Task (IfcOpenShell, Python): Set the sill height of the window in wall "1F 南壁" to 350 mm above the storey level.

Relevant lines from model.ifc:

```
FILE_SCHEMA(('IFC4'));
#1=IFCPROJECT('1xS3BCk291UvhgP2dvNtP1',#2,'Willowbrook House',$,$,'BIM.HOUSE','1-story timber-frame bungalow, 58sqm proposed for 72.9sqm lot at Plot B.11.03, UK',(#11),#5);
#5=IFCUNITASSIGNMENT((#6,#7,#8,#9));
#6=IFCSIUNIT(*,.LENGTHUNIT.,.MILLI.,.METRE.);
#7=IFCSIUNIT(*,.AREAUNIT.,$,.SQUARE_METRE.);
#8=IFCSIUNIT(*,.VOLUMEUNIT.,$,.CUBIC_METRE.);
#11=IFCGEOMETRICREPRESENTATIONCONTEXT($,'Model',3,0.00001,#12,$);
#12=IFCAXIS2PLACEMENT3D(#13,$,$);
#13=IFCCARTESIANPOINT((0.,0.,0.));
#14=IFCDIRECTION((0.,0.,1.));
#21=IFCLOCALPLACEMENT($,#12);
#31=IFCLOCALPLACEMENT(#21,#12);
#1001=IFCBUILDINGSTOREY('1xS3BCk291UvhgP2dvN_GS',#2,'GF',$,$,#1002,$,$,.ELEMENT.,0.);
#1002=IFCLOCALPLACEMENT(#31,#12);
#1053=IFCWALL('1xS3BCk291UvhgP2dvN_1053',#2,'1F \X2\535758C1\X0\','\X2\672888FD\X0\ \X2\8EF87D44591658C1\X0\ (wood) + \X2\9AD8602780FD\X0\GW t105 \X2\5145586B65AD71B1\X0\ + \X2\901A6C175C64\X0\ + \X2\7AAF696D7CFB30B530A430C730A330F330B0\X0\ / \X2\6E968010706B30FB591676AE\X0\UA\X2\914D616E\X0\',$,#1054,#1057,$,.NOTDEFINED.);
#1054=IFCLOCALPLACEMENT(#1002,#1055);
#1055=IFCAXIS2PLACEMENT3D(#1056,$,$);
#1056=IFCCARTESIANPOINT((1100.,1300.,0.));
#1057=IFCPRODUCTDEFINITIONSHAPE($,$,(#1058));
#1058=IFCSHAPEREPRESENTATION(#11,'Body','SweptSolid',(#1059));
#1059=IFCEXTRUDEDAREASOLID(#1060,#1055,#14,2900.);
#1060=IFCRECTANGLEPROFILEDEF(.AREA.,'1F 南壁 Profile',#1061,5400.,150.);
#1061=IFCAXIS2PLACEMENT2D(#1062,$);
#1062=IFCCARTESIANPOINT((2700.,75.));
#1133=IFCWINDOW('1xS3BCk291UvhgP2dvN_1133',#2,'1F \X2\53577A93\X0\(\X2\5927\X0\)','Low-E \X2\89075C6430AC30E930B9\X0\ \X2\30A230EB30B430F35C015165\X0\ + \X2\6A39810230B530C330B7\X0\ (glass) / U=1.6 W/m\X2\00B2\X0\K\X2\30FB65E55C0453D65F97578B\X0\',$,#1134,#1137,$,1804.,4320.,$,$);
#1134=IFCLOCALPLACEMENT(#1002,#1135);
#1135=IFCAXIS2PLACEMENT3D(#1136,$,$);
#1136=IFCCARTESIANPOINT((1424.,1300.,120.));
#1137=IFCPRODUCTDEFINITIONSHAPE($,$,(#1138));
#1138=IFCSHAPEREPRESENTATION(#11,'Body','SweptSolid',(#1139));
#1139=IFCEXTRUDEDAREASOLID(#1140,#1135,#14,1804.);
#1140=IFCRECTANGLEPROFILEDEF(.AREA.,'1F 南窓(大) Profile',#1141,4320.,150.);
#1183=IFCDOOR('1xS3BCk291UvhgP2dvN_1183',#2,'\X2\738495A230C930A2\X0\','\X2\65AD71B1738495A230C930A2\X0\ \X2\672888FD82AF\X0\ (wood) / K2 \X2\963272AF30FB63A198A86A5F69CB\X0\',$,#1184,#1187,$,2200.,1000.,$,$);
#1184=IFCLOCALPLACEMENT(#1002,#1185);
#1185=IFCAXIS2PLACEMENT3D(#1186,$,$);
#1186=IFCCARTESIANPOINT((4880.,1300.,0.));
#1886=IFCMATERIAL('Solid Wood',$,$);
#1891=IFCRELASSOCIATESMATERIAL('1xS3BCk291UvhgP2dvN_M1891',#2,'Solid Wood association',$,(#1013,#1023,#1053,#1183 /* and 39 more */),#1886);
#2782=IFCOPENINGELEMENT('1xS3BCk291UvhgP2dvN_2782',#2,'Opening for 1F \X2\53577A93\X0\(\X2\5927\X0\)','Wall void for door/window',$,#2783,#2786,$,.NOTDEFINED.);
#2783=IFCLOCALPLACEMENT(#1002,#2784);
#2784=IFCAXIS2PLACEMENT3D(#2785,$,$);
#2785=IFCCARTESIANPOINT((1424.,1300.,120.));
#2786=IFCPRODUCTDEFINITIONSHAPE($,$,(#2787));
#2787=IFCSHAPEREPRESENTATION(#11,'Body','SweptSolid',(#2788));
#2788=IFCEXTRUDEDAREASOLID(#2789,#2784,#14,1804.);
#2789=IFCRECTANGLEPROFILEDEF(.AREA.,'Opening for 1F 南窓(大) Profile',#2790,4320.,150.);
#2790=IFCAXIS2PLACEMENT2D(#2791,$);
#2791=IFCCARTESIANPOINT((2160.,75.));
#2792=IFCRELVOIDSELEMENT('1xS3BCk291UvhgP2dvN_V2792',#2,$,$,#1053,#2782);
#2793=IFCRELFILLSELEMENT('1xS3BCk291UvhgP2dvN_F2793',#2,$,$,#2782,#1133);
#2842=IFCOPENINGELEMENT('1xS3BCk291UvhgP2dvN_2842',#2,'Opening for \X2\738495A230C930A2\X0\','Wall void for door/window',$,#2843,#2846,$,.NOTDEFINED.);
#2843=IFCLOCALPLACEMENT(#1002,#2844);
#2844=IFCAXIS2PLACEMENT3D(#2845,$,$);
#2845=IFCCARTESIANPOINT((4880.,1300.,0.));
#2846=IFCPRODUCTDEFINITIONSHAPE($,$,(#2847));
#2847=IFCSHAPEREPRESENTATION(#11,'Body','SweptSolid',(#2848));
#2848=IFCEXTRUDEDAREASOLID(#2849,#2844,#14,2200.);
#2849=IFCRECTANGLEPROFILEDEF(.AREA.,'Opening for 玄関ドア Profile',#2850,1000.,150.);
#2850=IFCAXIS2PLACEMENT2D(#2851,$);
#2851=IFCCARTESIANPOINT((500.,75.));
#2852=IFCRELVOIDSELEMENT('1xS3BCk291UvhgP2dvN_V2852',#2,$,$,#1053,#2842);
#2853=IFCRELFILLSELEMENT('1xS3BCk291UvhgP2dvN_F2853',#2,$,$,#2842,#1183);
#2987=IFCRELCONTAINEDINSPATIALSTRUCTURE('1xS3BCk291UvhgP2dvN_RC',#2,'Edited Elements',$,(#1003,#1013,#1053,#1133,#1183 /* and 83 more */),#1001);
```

```python
import numpy as np
import ifcopenshell
import ifcopenshell.api.geometry
import ifcopenshell.geom
import ifcopenshell.util.element
import ifcopenshell.util.placement
import ifcopenshell.util.shape
import ifcopenshell.util.unit

model = ifcopenshell.open("model.ifc")
unit_scale = ifcopenshell.util.unit.calculate_unit_scale(model)

window = model.by_id(1133)
opening = window.FillsVoids[0].RelatingOpeningElement
storey = ifcopenshell.util.element.get_container(window, ifc_class="IfcBuildingStorey")
level = ifcopenshell.util.placement.get_local_placement(storey.ObjectPlacement)[2, 3]

# The opening's origin need not be at the sill, so measure its lowest point.
shape = ifcopenshell.geom.create_shape(ifcopenshell.geom.settings(), opening)
bottom = ifcopenshell.util.shape.get_shape_bottom_elevation(shape, shape.geometry) / unit_scale
dz = level + 0.35 / unit_scale - bottom

shift = np.array([0.0, 0.0, dz])
# The window is not placed relative to its opening, so move both.
for product in (opening, window):
    matrix = ifcopenshell.util.placement.get_local_placement(product.ObjectPlacement)
    matrix[:3, 3] += shift
    ifcopenshell.api.geometry.edit_object_placement(model, product=product, matrix=matrix, is_si=False)

print(f"moved by {dz * unit_scale:+.3f} m")

model.write("model_rev.ifc")
```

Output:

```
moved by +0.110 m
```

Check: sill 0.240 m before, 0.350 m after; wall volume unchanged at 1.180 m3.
